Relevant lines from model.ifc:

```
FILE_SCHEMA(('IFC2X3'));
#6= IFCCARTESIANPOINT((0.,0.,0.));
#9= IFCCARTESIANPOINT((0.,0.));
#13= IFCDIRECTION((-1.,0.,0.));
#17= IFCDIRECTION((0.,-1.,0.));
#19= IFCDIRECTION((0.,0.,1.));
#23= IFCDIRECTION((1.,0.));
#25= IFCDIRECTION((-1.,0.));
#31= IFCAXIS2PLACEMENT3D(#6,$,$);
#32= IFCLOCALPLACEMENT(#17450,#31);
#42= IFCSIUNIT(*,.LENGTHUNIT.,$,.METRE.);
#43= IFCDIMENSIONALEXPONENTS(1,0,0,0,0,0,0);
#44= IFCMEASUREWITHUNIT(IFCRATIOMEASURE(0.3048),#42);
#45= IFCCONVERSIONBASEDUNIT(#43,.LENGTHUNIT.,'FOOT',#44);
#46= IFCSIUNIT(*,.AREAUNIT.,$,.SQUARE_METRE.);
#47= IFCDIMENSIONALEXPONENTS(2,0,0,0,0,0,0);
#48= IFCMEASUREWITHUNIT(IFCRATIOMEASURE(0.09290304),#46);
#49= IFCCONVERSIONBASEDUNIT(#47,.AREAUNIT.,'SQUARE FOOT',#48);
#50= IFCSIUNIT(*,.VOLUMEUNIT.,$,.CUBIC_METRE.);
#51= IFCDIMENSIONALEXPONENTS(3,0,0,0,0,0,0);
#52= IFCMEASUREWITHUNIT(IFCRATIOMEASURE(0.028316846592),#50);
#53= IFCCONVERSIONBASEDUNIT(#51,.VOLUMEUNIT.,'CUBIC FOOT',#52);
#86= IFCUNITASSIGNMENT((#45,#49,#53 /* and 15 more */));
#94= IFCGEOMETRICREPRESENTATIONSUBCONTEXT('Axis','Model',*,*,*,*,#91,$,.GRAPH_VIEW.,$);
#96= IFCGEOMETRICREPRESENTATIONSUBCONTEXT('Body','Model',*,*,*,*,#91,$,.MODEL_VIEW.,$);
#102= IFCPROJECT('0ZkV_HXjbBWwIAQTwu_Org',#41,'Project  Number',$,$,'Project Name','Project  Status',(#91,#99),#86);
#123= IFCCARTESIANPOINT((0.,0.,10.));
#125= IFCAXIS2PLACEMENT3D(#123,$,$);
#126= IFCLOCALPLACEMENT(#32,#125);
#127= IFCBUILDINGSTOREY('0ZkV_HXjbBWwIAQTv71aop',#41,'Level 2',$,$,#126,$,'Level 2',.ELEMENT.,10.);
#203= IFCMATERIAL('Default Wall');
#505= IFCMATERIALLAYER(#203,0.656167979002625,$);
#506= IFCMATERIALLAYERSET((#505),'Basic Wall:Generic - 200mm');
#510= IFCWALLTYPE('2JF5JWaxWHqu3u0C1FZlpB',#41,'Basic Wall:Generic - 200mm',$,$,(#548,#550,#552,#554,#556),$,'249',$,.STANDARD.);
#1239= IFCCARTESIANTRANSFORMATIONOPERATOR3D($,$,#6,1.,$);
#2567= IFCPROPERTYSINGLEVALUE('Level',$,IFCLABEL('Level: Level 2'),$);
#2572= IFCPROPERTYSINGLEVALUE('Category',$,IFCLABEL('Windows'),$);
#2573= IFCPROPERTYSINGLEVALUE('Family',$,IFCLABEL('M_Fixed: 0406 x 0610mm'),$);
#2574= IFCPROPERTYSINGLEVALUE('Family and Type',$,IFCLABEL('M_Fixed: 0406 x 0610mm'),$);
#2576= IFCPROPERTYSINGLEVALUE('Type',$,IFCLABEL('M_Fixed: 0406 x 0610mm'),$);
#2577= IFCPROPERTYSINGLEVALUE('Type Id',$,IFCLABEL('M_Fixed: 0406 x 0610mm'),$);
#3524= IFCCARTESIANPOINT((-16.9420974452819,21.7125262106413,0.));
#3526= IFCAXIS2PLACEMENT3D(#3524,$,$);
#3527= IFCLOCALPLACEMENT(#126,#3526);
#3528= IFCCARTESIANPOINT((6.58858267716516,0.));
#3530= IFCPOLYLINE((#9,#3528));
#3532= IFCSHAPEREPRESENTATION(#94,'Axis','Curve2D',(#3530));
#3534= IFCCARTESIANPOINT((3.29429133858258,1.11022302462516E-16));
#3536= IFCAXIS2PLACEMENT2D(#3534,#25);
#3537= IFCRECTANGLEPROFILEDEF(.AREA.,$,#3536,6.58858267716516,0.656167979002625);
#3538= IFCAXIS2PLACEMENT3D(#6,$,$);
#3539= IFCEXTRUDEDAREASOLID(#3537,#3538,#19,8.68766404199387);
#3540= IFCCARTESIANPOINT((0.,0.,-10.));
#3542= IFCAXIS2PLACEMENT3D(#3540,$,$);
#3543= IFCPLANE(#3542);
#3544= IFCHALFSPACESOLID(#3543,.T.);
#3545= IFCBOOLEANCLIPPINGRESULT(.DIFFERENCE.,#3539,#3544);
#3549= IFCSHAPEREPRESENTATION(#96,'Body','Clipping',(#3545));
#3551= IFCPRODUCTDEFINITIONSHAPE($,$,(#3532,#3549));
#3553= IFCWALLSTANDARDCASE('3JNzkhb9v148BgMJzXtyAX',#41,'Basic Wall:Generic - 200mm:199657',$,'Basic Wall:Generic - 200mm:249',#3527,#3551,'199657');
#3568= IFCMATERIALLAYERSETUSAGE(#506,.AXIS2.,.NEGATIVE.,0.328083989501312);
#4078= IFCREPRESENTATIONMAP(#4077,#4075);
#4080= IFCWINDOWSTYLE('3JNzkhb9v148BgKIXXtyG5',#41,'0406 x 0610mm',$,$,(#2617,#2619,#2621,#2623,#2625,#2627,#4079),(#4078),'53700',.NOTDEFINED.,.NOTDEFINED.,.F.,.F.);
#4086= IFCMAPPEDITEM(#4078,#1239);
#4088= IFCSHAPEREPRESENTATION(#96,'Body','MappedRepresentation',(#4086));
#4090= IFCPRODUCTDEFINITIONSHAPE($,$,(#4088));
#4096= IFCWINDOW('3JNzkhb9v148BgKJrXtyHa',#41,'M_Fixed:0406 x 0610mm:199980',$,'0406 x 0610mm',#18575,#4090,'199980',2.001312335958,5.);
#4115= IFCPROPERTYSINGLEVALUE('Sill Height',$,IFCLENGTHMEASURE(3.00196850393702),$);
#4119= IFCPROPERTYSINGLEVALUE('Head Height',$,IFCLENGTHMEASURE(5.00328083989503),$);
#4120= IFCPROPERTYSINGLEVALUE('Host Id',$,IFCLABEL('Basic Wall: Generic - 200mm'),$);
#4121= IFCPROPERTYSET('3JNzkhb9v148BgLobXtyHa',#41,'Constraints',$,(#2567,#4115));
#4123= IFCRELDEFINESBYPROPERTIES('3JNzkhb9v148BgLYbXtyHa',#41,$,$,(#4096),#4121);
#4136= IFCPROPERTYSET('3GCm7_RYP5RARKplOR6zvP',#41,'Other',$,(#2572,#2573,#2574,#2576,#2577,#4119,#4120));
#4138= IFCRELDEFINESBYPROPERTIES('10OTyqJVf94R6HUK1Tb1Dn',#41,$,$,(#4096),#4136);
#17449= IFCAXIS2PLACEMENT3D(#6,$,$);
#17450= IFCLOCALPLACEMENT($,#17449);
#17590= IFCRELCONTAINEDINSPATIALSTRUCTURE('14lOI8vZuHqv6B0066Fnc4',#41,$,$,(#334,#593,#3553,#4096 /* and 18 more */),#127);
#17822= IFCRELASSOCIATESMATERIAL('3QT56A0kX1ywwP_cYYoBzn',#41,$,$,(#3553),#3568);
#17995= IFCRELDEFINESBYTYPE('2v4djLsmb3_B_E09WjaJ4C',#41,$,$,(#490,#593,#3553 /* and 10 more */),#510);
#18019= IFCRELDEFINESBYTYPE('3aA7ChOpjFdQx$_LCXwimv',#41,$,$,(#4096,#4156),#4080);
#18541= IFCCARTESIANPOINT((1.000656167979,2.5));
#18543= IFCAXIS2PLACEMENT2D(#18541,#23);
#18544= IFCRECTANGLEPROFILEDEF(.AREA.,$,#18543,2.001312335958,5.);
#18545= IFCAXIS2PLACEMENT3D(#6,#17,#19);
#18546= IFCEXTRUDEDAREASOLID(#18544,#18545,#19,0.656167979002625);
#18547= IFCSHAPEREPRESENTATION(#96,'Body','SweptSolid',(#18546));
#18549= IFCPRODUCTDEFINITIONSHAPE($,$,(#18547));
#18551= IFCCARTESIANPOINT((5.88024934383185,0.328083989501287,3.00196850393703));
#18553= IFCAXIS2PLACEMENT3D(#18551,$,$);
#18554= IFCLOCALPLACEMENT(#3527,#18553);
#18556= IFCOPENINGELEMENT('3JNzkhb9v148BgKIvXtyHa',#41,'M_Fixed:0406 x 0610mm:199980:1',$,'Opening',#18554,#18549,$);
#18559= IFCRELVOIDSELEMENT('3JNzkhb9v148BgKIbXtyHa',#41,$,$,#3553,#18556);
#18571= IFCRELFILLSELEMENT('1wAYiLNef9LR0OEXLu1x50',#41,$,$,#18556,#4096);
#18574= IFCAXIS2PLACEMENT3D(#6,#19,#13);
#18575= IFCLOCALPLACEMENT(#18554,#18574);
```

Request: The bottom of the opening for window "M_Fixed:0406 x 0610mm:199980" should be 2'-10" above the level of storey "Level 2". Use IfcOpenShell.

```python
import numpy as np
import ifcopenshell
import ifcopenshell.api.geometry
import ifcopenshell.api.pset
import ifcopenshell.geom
import ifcopenshell.util.element
import ifcopenshell.util.placement
import ifcopenshell.util.shape
import ifcopenshell.util.unit

model = ifcopenshell.open("model.ifc")
unit_scale = ifcopenshell.util.unit.calculate_unit_scale(model)

window = model.by_id(4096)
opening = window.FillsVoids[0].RelatingOpeningElement
storey = ifcopenshell.util.element.get_container(window, ifc_class="IfcBuildingStorey")
level = ifcopenshell.util.placement.get_local_placement(storey.ObjectPlacement)[2, 3]

# The opening's origin need not be at the sill, so measure its lowest point.
shape = ifcopenshell.geom.create_shape(ifcopenshell.geom.settings(), opening)
bottom = ifcopenshell.util.shape.get_shape_bottom_elevation(shape, shape.geometry) / unit_scale
dz = level + 34 * 0.0254 / unit_scale - bottom

shift = np.array([0.0, 0.0, dz])
# The window is placed relative to its opening, so it follows when the opening moves.
matrix = ifcopenshell.util.placement.get_local_placement(opening.ObjectPlacement)
matrix[:3, 3] += shift
ifcopenshell.api.geometry.edit_object_placement(
    model, product=opening, matrix=matrix, is_si=False, should_transform_children=True
)

# Keep the stored heights in step.
pset = model.by_id(ifcopenshell.util.element.get_pset(window, "Constraints", should_inherit=False)["id"])
ifcopenshell.api.pset.edit_pset(model, pset=pset, properties={
    "Sill Height": model.create_entity("IfcLengthMeasure", ifcopenshell.util.element.get_pset(window, "Constraints", "Sill Height") + dz),
})
pset = model.by_id(ifcopenshell.util.element.get_pset(window, "Other", should_inherit=False)["id"])
ifcopenshell.api.pset.edit_pset(model, pset=pset, properties={
    "Head Height": model.create_entity("IfcLengthMeasure", ifcopenshell.util.element.get_pset(window, "Other", "Head Height") + dz),
})

print(f"moved by {dz * unit_scale:+.3f} m")

model.write("model_updated.ifc")
```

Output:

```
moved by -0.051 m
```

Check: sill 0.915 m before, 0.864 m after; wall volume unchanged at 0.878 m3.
